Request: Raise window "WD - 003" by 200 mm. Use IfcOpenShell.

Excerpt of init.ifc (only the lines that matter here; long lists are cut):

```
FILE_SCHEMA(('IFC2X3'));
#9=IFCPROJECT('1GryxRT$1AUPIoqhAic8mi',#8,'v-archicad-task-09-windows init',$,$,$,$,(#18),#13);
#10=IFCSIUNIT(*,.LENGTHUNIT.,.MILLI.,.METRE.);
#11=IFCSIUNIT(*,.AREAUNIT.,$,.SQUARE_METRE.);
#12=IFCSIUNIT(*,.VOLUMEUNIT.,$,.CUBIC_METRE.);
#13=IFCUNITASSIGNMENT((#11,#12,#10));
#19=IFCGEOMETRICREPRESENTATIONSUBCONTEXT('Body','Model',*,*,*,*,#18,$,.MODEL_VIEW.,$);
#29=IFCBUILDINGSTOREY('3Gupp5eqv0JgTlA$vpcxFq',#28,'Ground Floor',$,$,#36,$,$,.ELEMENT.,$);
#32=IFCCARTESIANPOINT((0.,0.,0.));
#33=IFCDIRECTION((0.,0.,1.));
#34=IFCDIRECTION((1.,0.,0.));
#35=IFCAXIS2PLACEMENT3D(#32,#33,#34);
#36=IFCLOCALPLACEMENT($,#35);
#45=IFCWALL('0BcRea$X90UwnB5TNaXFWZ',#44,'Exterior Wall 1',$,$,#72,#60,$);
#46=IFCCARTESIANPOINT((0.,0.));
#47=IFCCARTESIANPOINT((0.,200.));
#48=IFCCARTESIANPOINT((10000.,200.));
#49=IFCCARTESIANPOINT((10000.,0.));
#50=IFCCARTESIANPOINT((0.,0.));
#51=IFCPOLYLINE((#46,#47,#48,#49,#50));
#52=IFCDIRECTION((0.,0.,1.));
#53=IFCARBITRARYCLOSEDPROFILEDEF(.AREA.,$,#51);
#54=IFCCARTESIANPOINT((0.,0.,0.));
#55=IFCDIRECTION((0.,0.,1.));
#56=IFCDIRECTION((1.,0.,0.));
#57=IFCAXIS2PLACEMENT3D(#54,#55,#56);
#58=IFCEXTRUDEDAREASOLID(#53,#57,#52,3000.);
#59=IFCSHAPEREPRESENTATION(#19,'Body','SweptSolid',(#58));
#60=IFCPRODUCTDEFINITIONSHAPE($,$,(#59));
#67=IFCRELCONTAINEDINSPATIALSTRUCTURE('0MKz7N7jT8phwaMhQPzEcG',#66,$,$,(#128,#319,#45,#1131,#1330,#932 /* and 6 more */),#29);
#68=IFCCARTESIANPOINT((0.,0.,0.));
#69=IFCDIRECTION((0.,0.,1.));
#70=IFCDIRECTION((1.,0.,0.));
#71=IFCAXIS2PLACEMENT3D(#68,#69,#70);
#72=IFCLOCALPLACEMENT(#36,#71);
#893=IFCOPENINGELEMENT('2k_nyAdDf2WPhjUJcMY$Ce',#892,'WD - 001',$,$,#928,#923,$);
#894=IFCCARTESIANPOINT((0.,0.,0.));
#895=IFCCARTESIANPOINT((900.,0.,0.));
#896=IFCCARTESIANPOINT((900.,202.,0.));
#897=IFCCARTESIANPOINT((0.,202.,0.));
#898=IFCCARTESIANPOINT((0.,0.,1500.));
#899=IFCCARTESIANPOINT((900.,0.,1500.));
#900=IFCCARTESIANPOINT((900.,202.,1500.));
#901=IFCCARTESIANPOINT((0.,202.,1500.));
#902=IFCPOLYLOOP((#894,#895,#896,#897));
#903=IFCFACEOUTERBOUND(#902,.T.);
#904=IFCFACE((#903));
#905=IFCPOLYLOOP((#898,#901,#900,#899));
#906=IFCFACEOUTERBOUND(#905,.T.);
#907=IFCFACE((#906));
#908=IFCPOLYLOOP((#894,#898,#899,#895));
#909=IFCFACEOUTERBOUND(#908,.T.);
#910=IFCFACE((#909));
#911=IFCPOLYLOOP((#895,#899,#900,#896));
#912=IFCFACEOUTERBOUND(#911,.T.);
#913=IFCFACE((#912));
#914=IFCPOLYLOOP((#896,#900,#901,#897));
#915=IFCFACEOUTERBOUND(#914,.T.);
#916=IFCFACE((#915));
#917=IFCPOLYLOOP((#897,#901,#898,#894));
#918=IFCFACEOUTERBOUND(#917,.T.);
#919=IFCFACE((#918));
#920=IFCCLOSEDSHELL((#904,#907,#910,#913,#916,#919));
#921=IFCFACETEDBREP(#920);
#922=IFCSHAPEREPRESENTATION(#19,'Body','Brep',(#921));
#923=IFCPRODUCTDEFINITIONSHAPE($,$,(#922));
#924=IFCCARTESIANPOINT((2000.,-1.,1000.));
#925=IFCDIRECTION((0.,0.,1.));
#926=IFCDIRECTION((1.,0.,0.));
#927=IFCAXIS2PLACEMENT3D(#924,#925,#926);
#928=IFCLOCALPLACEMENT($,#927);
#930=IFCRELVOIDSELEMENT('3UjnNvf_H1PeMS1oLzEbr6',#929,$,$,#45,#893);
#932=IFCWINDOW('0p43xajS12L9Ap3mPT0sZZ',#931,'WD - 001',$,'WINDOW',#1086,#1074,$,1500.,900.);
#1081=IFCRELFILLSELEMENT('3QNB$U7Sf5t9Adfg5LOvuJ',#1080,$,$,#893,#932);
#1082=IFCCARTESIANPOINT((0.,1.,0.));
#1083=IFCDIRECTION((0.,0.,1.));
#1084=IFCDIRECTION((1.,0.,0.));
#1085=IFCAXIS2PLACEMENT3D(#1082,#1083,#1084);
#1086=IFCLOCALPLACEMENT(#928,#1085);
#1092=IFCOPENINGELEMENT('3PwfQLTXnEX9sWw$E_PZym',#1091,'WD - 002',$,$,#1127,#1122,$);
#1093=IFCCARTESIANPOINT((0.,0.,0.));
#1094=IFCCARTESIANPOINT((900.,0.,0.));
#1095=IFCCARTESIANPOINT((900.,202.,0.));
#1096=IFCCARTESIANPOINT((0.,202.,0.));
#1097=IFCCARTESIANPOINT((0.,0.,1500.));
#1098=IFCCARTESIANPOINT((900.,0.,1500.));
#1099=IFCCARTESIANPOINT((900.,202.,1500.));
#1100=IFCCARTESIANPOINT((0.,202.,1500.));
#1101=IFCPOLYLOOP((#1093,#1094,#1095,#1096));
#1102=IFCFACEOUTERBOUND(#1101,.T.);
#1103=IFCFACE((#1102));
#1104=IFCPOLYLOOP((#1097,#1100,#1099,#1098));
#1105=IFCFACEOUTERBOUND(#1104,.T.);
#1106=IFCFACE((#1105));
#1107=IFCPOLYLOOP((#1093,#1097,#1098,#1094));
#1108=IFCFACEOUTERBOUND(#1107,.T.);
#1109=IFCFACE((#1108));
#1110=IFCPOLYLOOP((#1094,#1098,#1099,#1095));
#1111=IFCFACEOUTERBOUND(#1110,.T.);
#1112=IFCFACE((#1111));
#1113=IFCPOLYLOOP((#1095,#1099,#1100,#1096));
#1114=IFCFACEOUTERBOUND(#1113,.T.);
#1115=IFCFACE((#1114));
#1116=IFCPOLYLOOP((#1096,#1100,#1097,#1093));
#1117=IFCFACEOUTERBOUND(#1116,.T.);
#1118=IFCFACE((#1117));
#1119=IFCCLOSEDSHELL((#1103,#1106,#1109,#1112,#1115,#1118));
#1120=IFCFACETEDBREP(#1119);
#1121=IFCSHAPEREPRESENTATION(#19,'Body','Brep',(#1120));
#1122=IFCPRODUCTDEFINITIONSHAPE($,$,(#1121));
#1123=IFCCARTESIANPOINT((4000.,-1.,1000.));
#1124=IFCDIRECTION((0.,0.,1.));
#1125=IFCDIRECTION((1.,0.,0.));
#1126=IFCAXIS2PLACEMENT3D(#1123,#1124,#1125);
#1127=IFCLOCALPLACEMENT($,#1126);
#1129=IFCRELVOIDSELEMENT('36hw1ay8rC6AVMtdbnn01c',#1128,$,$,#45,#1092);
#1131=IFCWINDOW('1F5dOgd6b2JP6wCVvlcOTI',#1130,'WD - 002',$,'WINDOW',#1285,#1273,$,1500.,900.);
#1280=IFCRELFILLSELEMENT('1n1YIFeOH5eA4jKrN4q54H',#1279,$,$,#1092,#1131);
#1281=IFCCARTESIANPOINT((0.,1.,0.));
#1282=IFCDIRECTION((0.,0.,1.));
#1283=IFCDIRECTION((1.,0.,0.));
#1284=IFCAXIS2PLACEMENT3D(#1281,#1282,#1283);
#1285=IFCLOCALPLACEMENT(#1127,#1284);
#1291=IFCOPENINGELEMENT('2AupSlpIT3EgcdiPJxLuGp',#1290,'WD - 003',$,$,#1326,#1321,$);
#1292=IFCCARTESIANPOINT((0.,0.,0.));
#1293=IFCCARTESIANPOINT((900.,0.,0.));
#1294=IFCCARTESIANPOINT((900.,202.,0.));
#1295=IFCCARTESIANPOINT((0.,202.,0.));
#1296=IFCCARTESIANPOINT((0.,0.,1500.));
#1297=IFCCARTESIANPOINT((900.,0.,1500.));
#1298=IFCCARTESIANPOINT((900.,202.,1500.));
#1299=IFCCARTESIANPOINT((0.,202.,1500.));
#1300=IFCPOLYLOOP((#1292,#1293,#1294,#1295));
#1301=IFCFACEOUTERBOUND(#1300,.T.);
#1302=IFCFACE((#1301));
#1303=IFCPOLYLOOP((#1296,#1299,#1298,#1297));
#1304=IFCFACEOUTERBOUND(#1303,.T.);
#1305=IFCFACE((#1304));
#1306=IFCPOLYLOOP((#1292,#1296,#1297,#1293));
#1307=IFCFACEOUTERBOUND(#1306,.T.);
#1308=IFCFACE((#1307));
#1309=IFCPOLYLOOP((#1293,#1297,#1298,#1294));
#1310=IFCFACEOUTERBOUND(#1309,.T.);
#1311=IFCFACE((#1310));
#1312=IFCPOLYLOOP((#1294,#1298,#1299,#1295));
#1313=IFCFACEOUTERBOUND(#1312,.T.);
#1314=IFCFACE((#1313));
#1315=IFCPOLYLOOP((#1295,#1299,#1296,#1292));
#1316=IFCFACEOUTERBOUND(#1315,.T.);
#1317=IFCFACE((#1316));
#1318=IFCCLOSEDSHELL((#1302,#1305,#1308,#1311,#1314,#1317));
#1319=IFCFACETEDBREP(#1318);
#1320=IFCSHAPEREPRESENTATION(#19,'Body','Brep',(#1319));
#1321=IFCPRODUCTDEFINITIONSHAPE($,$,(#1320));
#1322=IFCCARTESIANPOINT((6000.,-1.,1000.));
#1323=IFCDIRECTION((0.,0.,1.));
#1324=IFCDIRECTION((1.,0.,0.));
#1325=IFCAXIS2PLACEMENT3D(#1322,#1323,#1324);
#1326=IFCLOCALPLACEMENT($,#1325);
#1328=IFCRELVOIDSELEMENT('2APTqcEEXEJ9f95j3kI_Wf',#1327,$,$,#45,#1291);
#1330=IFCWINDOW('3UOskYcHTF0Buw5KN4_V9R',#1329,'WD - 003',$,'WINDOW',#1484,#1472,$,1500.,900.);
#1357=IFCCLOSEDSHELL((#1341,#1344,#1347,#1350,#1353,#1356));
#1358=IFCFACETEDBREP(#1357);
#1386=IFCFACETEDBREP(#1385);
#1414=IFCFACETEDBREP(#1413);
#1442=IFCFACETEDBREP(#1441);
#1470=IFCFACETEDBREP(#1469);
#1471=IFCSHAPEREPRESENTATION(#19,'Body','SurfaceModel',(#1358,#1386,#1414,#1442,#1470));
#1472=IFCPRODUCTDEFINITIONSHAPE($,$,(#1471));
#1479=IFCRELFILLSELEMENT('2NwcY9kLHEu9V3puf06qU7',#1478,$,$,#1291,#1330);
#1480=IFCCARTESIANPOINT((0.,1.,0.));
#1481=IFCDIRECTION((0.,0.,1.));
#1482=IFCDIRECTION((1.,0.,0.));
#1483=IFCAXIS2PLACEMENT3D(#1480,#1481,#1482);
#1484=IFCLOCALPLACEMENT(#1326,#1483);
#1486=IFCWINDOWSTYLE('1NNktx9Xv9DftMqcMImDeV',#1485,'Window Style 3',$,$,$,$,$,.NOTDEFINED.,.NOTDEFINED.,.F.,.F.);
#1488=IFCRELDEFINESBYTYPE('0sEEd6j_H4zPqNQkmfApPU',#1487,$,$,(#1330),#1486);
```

```python
import numpy as np
import ifcopenshell
import ifcopenshell.api.geometry
import ifcopenshell.util.placement
import ifcopenshell.util.unit

model = ifcopenshell.open("init.ifc")
unit_scale = ifcopenshell.util.unit.calculate_unit_scale(model)

window = model.by_guid("3UOskYcHTF0Buw5KN4_V9R")
opening = window.FillsVoids[0].RelatingOpeningElement
dz = 200.0

shift = np.array([0.0, 0.0, dz])
# The window is placed relative to its opening, so it follows when the opening moves.
matrix = ifcopenshell.util.placement.get_local_placement(opening.ObjectPlacement)
matrix[:3, 3] += shift
ifcopenshell.api.geometry.edit_object_placement(
    model, product=opening, matrix=matrix, is_si=False, should_transform_children=True
)

print(f"moved by {dz * unit_scale:+.3f} m")

model.write("init_edited.ifc")
```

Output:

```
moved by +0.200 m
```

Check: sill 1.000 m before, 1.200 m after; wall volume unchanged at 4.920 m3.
